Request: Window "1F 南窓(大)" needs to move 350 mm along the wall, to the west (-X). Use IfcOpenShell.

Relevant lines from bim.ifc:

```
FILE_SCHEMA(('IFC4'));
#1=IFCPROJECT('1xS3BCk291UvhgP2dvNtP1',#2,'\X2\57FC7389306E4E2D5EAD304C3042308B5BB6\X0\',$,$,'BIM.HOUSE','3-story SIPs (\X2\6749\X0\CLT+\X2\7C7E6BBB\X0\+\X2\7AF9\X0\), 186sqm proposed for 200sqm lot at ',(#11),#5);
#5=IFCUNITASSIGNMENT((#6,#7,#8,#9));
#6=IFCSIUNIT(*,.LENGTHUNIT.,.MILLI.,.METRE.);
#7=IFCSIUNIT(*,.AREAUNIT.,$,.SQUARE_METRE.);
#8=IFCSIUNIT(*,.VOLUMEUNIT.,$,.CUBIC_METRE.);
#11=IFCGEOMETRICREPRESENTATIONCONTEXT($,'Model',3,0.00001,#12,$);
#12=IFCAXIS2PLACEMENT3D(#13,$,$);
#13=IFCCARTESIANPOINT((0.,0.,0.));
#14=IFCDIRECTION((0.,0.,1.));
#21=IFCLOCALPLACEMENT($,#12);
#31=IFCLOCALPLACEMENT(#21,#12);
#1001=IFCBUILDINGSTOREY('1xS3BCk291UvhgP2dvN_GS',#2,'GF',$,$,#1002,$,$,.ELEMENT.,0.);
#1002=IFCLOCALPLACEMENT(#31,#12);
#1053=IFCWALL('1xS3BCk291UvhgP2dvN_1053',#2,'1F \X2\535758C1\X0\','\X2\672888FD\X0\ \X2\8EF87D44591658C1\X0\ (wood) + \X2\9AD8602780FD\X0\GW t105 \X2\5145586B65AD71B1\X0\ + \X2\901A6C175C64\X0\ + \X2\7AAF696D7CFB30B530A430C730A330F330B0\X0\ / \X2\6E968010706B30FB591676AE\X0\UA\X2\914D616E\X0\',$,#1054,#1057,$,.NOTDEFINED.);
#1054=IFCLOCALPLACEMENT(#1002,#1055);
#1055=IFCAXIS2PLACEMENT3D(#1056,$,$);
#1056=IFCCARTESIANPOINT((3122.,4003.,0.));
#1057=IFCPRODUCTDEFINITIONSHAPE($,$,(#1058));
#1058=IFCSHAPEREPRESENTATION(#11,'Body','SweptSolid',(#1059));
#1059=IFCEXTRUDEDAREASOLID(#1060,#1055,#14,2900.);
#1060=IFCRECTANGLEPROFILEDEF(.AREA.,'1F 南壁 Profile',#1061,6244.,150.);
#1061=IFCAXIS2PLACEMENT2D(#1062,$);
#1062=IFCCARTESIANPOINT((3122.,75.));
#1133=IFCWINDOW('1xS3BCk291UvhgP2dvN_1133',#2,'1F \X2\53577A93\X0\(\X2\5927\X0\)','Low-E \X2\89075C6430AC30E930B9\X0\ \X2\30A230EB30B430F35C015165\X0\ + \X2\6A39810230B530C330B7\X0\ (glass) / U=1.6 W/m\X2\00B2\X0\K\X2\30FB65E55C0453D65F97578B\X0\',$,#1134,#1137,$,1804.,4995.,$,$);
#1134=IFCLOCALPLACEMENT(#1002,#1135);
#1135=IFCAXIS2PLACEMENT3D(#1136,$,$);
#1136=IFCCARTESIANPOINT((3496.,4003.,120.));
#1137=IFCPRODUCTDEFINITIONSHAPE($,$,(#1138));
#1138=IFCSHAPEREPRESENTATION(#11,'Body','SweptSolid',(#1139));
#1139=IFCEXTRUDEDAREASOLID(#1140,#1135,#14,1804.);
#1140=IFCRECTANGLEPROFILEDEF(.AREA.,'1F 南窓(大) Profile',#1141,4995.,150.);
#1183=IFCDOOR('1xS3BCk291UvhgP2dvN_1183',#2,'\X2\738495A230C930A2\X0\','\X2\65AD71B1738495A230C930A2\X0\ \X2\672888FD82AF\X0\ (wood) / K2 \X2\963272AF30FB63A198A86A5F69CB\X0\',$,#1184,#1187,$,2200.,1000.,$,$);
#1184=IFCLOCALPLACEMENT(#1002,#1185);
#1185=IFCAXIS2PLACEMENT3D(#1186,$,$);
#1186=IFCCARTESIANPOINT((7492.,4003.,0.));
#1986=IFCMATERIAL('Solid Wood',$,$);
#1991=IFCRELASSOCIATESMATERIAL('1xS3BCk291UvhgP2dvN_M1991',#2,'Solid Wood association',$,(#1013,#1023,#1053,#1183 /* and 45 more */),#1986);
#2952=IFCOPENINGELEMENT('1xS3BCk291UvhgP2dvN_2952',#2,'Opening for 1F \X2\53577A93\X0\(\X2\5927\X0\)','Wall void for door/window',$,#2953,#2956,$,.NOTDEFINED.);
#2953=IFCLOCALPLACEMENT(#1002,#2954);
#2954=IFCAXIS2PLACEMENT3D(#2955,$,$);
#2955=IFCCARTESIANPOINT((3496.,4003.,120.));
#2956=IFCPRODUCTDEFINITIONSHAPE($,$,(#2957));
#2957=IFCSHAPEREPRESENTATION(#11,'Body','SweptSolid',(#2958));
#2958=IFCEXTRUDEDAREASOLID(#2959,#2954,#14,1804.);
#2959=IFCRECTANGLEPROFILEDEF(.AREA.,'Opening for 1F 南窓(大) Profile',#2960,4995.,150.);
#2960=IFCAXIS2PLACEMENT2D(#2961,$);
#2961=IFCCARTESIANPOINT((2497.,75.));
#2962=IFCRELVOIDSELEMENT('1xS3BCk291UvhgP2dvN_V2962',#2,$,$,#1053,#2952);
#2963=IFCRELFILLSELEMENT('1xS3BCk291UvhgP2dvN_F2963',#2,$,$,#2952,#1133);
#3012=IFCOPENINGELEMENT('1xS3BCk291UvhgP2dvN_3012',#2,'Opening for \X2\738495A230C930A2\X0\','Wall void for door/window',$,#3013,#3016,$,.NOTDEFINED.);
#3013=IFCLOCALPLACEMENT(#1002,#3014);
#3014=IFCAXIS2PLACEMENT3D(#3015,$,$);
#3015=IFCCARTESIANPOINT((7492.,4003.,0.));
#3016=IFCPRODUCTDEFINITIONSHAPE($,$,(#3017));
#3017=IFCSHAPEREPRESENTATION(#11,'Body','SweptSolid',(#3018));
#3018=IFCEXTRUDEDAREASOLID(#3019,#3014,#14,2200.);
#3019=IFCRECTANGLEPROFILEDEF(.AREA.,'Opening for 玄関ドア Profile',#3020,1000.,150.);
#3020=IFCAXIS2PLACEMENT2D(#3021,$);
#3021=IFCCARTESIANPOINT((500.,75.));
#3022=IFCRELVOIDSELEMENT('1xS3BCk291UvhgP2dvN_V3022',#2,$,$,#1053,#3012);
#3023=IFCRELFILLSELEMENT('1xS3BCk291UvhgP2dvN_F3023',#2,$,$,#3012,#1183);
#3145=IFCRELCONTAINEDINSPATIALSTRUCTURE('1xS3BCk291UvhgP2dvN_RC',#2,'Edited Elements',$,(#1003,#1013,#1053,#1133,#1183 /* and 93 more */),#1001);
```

```python
import ifcopenshell
import ifcopenshell.api.geometry
import ifcopenshell.util.placement

model = ifcopenshell.open("bim.ifc")

window = model.by_id(1133)
opening = window.FillsVoids[0].RelatingOpeningElement
wall = opening.VoidsElements[0].RelatingBuildingElement

wall_matrix = ifcopenshell.util.placement.get_local_placement(wall.ObjectPlacement)
shift = wall_matrix[:3, 0] * -350.0
before = ifcopenshell.util.placement.get_local_placement(window.ObjectPlacement)[:3, 3].copy()

# The window is not placed relative to its opening, so move both.
for product in (opening, window):
    matrix = ifcopenshell.util.placement.get_local_placement(product.ObjectPlacement)
    matrix[:3, 3] += shift
    ifcopenshell.api.geometry.edit_object_placement(model, product=product, matrix=matrix, is_si=False)

after = ifcopenshell.util.placement.get_local_placement(window.ObjectPlacement)[:3, 3]
print("window moved by", (after - before).round(3) + 0.0)

model.write("bim_v2.ifc")
```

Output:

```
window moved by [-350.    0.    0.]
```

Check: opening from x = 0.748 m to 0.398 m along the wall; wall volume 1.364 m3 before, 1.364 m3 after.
